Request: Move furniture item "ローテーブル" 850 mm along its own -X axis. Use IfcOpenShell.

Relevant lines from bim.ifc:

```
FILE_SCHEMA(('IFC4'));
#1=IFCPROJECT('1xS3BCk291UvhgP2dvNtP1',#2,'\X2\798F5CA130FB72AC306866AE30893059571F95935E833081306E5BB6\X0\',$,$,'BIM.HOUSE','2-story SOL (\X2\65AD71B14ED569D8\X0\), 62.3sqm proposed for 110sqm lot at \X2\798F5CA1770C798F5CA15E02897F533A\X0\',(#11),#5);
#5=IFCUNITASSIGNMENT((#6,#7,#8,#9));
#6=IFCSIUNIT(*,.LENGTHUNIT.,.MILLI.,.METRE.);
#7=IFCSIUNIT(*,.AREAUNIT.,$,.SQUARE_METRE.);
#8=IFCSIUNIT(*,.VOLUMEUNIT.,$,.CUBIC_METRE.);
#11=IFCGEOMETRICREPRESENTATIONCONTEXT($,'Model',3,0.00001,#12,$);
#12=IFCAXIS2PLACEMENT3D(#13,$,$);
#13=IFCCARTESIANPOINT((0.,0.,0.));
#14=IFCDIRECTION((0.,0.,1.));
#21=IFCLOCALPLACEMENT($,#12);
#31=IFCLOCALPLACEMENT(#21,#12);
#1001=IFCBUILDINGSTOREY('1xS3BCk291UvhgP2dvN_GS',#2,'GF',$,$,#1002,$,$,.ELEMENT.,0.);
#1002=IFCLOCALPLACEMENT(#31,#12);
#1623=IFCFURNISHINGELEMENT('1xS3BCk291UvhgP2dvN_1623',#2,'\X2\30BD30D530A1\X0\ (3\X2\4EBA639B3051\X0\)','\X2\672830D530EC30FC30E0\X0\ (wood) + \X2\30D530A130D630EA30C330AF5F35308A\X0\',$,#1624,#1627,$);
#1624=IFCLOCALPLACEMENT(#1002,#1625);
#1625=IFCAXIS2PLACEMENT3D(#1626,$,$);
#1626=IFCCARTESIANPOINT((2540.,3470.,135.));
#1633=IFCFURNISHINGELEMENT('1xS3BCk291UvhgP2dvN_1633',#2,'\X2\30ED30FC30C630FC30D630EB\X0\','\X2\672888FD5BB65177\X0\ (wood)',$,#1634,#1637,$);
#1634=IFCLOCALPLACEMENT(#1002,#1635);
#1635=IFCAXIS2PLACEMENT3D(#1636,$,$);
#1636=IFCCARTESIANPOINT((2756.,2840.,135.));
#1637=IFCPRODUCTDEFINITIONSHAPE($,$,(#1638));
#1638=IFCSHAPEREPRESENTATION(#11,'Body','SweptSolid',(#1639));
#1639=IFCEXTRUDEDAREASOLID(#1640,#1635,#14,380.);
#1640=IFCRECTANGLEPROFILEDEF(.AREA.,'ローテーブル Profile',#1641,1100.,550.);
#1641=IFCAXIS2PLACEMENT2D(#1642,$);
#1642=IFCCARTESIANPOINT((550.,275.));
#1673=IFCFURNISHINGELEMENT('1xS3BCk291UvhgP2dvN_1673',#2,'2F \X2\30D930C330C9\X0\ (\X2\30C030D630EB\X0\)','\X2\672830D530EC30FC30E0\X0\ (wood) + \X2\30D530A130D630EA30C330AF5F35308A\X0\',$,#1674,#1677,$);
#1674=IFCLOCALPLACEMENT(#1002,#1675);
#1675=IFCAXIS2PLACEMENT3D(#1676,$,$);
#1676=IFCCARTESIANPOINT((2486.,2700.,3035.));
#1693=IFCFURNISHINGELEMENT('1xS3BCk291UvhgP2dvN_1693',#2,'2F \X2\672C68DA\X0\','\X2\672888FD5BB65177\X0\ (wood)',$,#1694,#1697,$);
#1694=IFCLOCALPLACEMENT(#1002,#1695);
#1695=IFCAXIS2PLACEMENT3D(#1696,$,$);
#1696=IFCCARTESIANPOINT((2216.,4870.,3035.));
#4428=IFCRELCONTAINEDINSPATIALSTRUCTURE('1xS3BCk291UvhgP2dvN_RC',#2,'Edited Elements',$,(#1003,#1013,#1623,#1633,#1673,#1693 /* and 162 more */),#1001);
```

```python
import ifcopenshell
import ifcopenshell.api.geometry
import ifcopenshell.util.placement
import ifcopenshell.util.unit

model = ifcopenshell.open("bim.ifc")
unit_scale = ifcopenshell.util.unit.calculate_unit_scale(model)

item = model.by_id(1633)
matrix = ifcopenshell.util.placement.get_local_placement(item.ObjectPlacement)
matrix[:3, 3] -= matrix[:3, 0] * 0.85 / unit_scale
ifcopenshell.api.geometry.edit_object_placement(model, product=item, matrix=matrix, is_si=False)

print(ifcopenshell.util.placement.get_local_placement(item.ObjectPlacement).round(3) + 0.0)

model.write("bim_rev.ifc")
```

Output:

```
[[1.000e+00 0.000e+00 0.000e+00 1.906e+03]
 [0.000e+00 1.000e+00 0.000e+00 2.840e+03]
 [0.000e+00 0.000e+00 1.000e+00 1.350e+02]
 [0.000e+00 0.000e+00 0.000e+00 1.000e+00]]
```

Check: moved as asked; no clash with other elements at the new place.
